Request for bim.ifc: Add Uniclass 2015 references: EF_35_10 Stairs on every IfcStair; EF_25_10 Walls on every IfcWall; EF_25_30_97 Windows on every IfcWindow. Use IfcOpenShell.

First a look at what the model holds.

```python
import ifcopenshell

model = ifcopenshell.open("bim.ifc")
print(model.schema)
print("classifications:", [c.Name for c in model.by_type("IfcClassification")])
for ifc_class in ("IfcDoor", "IfcRoof", "IfcStair", "IfcWall", "IfcWindow"):
    print(ifc_class, len(model.by_type(ifc_class)))
```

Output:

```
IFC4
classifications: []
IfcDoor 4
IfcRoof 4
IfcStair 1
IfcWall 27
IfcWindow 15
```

```python
import ifcopenshell
import ifcopenshell.api.classification

model = ifcopenshell.open("bim.ifc")

system = ifcopenshell.api.classification.add_classification(model, classification="Uniclass 2015")

codes = {
    "IfcStair": ("EF_35_10", "Stairs"),
    "IfcWall": ("EF_25_10", "Walls"),
    "IfcWindow": ("EF_25_30_97", "Windows"),
}
for ifc_class, (code, name) in codes.items():
    products = model.by_type(ifc_class)
    ifcopenshell.api.classification.add_reference(
        model, products=products, classification=system, identification=code, name=name
    )
    print(code, len(products))

model.write("bim_v2.ifc")
```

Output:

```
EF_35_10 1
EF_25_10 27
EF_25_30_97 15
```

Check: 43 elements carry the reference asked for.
